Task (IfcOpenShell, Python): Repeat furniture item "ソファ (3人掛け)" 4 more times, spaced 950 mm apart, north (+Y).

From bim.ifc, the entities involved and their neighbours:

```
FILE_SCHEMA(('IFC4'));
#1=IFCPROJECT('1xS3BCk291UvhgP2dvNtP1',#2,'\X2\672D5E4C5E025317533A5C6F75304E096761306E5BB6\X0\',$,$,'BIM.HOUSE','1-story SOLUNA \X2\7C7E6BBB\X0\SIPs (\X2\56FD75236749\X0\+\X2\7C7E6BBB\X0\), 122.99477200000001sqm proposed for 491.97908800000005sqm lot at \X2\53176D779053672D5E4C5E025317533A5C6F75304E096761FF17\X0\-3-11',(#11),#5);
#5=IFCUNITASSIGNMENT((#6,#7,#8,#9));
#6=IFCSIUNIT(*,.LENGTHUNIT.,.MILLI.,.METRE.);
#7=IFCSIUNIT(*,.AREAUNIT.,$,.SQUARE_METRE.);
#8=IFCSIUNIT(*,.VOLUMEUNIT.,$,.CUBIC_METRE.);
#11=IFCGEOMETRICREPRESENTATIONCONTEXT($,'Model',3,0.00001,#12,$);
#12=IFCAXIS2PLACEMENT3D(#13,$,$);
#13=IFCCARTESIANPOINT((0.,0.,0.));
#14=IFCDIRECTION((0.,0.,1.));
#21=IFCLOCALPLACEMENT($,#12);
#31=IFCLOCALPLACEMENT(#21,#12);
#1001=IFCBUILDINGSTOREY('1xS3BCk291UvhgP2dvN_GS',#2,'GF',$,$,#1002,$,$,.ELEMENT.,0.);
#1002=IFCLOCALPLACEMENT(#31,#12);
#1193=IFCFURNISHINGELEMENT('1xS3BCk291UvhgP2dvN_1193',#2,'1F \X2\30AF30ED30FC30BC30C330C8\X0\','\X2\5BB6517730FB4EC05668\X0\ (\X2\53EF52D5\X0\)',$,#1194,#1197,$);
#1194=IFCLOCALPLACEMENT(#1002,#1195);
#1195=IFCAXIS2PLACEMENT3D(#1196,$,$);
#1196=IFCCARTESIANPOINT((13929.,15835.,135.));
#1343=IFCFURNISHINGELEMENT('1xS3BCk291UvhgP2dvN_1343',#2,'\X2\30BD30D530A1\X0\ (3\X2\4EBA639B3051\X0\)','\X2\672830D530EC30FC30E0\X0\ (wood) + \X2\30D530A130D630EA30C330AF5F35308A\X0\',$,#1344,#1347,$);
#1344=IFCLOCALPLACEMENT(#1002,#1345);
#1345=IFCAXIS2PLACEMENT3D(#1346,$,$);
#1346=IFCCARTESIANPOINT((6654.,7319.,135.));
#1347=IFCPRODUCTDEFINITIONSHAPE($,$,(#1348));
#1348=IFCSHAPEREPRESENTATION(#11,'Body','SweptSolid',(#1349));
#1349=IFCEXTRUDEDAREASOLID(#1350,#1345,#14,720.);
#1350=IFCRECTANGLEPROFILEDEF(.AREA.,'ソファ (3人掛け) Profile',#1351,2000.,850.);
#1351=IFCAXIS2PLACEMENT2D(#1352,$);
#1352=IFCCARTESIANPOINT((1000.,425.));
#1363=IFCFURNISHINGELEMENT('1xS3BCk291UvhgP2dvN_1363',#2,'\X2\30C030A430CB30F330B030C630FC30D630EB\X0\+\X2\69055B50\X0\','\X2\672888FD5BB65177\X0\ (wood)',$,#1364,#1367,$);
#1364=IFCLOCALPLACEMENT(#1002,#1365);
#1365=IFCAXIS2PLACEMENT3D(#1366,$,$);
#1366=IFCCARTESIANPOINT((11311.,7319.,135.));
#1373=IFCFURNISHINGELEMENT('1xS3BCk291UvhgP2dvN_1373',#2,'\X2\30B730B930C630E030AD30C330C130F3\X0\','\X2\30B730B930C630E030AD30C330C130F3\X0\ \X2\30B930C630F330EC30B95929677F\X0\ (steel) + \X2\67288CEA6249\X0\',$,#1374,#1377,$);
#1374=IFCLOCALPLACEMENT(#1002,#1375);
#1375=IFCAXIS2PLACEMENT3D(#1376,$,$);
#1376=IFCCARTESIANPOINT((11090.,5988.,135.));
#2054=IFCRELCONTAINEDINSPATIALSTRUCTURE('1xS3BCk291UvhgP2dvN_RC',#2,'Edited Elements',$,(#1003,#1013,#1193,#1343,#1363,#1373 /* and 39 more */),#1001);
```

```python
import numpy as np
import ifcopenshell
import ifcopenshell.api.geometry
import ifcopenshell.api.root
import ifcopenshell.util.element
import ifcopenshell.util.placement

model = ifcopenshell.open("bim.ifc")


def reuse_history(source, copy):
    """copy_class also copies each property set's owner history, people and application; keep the originals."""
    for rel in copy.IsDefinedBy:
        if rel.is_a("IfcRelDefinesByProperties") and (history := rel.RelatingPropertyDefinition.OwnerHistory):
            rel.RelatingPropertyDefinition.OwnerHistory = source.OwnerHistory
            ifcopenshell.util.element.remove_deep2(model, history)


source = model.by_guid("1xS3BCk291UvhgP2dvN_1343")
base = ifcopenshell.util.placement.get_local_placement(source.ObjectPlacement)
step = np.array([0.0, 1.0, 0.0]) * 950.0

for i in range(1, 5):
    copy = ifcopenshell.api.root.copy_class(model, product=source)
    copy.Representation = ifcopenshell.util.element.copy_deep(
        model, source.Representation, exclude=["IfcGeometricRepresentationContext", "IfcRepresentationMap"]
    )
    reuse_history(source, copy)
    matrix = base.copy()
    matrix[:3, 3] += i * step
    print("added at", matrix[:3, 3].round(3) + 0.0)
    ifcopenshell.api.geometry.edit_object_placement(model, product=copy, matrix=matrix, is_si=False)

model.write("bim_edited.ifc")
```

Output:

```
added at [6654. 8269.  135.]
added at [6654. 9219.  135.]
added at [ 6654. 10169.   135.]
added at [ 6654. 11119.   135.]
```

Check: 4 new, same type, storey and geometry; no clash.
